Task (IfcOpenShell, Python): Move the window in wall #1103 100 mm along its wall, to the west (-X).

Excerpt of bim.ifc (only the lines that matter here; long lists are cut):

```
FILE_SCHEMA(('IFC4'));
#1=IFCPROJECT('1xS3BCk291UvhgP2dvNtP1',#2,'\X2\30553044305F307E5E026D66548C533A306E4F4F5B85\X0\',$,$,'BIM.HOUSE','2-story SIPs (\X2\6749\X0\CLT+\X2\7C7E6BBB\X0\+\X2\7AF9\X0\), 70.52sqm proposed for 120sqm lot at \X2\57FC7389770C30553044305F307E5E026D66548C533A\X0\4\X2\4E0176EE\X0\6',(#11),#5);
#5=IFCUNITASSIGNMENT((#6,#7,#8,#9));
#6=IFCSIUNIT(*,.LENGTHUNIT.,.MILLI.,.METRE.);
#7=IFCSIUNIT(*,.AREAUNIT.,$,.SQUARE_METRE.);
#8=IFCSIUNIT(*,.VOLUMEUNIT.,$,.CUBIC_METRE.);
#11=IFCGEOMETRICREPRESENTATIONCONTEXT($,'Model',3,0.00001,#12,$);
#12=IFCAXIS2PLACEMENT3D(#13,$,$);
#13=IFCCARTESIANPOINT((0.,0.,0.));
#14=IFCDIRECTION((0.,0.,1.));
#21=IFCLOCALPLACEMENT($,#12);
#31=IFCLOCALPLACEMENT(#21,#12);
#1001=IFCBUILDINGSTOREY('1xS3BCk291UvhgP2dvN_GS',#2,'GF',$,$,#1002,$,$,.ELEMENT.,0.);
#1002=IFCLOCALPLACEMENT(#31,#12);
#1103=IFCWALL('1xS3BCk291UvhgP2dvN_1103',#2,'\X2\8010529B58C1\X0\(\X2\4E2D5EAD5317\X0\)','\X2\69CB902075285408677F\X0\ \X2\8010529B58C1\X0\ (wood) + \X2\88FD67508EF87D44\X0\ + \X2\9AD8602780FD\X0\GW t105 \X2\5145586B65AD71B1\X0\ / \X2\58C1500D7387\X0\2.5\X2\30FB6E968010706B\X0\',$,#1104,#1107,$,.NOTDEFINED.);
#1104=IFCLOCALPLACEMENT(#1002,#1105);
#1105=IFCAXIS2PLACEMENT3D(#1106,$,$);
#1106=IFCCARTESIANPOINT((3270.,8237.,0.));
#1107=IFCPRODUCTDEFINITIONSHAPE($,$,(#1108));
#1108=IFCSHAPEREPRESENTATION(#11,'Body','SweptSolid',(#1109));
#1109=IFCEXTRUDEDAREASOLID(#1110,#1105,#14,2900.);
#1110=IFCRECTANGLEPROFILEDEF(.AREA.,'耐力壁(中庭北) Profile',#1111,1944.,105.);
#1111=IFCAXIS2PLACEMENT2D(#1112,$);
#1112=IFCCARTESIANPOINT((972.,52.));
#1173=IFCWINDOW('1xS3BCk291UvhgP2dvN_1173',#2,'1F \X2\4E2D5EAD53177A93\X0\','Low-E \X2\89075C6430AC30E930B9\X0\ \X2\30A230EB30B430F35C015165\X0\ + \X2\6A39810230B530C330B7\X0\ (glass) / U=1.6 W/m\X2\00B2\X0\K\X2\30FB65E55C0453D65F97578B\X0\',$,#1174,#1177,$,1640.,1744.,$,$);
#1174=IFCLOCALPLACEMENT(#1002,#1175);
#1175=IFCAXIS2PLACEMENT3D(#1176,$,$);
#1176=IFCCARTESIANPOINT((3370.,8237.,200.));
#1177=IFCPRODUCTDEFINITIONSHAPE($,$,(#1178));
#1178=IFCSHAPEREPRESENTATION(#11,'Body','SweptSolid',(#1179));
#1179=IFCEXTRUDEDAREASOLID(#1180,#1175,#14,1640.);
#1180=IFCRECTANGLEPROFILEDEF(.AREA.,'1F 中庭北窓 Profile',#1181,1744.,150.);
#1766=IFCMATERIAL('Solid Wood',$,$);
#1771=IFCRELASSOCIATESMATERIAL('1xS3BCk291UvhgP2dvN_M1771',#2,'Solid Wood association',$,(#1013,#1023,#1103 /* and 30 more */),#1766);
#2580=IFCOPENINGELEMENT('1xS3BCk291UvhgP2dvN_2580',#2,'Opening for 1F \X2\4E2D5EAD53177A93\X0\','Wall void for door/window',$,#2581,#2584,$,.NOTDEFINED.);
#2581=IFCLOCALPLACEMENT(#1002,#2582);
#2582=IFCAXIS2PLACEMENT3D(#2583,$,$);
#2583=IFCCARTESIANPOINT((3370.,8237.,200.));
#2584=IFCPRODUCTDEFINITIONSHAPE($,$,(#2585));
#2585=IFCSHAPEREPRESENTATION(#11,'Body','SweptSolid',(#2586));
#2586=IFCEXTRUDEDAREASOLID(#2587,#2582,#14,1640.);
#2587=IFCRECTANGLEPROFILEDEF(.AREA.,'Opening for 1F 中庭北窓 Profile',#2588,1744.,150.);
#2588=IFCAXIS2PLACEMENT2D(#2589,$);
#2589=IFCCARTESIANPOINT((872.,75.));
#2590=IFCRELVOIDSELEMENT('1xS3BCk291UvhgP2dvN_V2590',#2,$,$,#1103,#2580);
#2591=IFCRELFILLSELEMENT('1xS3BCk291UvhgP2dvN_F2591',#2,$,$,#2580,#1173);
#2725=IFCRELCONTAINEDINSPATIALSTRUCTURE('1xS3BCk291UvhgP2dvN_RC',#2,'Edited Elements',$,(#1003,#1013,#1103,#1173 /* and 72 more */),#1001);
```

```python
import ifcopenshell
import ifcopenshell.api.geometry
import ifcopenshell.util.placement
import ifcopenshell.util.unit

model = ifcopenshell.open("bim.ifc")
unit_scale = ifcopenshell.util.unit.calculate_unit_scale(model)

window = model.by_guid("1xS3BCk291UvhgP2dvN_1173")
opening = window.FillsVoids[0].RelatingOpeningElement
wall = opening.VoidsElements[0].RelatingBuildingElement

wall_matrix = ifcopenshell.util.placement.get_local_placement(wall.ObjectPlacement)
shift = wall_matrix[:3, 0] * -0.1 / unit_scale
before = ifcopenshell.util.placement.get_local_placement(window.ObjectPlacement)[:3, 3].copy()

# The window is not placed relative to its opening, so move both.
for product in (opening, window):
    matrix = ifcopenshell.util.placement.get_local_placement(product.ObjectPlacement)
    matrix[:3, 3] += shift
    ifcopenshell.api.geometry.edit_object_placement(model, product=product, matrix=matrix, is_si=False)

after = ifcopenshell.util.placement.get_local_placement(window.ObjectPlacement)[:3, 3]
print("window moved by", (after - before).round(3) + 0.0)

model.write("bim_v2.ifc")
```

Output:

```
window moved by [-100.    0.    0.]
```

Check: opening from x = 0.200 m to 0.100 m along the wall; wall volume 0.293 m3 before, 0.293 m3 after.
